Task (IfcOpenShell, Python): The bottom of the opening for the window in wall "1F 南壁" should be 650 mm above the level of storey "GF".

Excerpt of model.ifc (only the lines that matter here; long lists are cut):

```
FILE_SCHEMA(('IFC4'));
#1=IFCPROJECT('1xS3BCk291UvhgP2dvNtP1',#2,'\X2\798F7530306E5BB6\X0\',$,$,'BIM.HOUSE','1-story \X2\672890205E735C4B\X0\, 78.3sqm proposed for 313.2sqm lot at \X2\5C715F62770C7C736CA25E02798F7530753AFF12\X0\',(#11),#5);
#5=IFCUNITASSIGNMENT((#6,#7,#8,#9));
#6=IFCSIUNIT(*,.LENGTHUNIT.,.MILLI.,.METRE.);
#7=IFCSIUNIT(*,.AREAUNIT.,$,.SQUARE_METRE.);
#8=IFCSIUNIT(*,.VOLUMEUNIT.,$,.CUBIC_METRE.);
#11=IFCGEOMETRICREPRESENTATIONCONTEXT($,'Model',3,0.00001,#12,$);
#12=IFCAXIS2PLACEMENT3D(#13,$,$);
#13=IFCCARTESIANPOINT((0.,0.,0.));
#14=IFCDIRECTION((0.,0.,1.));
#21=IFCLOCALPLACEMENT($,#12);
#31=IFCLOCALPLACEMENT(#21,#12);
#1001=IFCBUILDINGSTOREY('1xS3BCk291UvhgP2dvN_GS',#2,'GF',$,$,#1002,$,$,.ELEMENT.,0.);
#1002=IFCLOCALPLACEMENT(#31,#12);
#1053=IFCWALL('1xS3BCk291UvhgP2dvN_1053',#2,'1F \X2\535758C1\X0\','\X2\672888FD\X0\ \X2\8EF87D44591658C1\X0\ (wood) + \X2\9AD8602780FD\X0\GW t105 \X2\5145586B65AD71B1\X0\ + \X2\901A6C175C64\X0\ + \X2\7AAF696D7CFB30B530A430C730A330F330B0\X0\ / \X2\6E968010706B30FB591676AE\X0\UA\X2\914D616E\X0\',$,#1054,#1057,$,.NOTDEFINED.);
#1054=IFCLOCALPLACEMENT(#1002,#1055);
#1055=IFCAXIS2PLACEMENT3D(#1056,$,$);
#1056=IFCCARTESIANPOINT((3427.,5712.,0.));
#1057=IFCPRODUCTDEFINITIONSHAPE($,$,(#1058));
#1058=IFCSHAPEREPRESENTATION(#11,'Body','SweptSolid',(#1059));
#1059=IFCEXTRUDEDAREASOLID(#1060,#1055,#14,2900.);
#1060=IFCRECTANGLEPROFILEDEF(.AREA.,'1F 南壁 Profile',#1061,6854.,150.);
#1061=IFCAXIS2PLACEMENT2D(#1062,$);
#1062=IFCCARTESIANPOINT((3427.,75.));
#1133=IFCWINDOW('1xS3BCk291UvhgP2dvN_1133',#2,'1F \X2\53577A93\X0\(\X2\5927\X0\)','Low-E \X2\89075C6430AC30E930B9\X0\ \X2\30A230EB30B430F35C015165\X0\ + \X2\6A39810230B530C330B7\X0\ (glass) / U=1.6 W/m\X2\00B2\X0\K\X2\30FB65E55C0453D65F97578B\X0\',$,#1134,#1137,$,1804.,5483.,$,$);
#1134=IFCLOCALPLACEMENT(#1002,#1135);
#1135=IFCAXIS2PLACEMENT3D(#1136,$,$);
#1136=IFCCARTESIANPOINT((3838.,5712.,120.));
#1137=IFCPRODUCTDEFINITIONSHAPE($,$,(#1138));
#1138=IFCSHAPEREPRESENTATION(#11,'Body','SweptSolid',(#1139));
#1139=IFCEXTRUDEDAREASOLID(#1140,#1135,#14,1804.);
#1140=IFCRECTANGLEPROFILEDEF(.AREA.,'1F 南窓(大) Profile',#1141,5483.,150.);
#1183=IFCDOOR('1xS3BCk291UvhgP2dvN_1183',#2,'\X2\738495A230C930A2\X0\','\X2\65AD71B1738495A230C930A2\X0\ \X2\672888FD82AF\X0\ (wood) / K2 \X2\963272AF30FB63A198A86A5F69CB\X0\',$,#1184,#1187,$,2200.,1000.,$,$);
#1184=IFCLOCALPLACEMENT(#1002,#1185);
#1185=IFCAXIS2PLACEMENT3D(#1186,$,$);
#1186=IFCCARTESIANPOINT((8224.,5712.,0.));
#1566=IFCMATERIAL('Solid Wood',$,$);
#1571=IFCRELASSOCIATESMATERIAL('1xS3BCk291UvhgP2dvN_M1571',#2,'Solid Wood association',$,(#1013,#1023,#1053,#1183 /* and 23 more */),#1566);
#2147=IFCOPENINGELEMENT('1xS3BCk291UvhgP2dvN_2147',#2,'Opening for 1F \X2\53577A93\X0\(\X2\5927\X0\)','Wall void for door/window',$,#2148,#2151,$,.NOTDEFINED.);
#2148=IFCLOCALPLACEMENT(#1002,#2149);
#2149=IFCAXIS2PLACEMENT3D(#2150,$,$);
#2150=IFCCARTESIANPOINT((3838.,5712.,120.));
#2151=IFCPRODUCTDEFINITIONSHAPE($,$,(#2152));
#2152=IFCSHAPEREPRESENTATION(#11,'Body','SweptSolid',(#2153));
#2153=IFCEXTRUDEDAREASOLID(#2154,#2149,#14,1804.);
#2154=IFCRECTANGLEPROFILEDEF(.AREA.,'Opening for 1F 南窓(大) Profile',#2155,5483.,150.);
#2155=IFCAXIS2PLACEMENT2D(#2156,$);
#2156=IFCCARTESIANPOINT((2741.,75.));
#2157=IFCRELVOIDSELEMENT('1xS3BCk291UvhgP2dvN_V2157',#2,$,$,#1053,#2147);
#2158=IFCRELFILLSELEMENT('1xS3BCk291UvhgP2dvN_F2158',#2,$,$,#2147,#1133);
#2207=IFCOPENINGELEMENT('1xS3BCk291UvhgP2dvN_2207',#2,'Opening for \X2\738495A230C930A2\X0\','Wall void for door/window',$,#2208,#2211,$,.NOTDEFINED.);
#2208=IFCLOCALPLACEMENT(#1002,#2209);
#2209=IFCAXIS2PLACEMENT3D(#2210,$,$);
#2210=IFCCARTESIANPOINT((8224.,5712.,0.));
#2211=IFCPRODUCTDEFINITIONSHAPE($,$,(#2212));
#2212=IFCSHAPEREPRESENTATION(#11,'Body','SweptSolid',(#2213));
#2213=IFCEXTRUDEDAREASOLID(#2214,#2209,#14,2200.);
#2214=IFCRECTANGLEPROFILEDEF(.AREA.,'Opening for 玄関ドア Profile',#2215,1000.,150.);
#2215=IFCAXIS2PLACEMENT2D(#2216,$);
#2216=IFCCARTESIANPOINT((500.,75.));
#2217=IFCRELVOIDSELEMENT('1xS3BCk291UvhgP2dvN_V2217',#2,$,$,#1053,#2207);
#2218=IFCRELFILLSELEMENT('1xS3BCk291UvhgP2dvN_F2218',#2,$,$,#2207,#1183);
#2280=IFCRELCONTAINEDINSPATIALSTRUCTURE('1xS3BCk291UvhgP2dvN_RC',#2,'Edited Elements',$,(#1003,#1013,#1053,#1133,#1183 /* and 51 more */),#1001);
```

```python
import numpy as np
import ifcopenshell
import ifcopenshell.api.geometry
import ifcopenshell.geom
import ifcopenshell.util.element
import ifcopenshell.util.placement
import ifcopenshell.util.shape
import ifcopenshell.util.unit

model = ifcopenshell.open("model.ifc")
unit_scale = ifcopenshell.util.unit.calculate_unit_scale(model)

window = model.by_guid("1xS3BCk291UvhgP2dvN_1133")
opening = window.FillsVoids[0].RelatingOpeningElement
storey = ifcopenshell.util.element.get_container(window, ifc_class="IfcBuildingStorey")
level = ifcopenshell.util.placement.get_local_placement(storey.ObjectPlacement)[2, 3]

# The opening's origin need not be at the sill, so measure its lowest point.
shape = ifcopenshell.geom.create_shape(ifcopenshell.geom.settings(), opening)
bottom = ifcopenshell.util.shape.get_shape_bottom_elevation(shape, shape.geometry) / unit_scale
dz = level + 650.0 - bottom

shift = np.array([0.0, 0.0, dz])
# The window is not placed relative to its opening, so move both.
for product in (opening, window):
    matrix = ifcopenshell.util.placement.get_local_placement(product.ObjectPlacement)
    matrix[:3, 3] += shift
    ifcopenshell.api.geometry.edit_object_placement(model, product=product, matrix=matrix, is_si=False)

print(f"moved by {dz * unit_scale:+.3f} m")

model.write("model_edited.ifc")
```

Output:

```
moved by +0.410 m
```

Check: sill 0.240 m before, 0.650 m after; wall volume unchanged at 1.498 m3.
